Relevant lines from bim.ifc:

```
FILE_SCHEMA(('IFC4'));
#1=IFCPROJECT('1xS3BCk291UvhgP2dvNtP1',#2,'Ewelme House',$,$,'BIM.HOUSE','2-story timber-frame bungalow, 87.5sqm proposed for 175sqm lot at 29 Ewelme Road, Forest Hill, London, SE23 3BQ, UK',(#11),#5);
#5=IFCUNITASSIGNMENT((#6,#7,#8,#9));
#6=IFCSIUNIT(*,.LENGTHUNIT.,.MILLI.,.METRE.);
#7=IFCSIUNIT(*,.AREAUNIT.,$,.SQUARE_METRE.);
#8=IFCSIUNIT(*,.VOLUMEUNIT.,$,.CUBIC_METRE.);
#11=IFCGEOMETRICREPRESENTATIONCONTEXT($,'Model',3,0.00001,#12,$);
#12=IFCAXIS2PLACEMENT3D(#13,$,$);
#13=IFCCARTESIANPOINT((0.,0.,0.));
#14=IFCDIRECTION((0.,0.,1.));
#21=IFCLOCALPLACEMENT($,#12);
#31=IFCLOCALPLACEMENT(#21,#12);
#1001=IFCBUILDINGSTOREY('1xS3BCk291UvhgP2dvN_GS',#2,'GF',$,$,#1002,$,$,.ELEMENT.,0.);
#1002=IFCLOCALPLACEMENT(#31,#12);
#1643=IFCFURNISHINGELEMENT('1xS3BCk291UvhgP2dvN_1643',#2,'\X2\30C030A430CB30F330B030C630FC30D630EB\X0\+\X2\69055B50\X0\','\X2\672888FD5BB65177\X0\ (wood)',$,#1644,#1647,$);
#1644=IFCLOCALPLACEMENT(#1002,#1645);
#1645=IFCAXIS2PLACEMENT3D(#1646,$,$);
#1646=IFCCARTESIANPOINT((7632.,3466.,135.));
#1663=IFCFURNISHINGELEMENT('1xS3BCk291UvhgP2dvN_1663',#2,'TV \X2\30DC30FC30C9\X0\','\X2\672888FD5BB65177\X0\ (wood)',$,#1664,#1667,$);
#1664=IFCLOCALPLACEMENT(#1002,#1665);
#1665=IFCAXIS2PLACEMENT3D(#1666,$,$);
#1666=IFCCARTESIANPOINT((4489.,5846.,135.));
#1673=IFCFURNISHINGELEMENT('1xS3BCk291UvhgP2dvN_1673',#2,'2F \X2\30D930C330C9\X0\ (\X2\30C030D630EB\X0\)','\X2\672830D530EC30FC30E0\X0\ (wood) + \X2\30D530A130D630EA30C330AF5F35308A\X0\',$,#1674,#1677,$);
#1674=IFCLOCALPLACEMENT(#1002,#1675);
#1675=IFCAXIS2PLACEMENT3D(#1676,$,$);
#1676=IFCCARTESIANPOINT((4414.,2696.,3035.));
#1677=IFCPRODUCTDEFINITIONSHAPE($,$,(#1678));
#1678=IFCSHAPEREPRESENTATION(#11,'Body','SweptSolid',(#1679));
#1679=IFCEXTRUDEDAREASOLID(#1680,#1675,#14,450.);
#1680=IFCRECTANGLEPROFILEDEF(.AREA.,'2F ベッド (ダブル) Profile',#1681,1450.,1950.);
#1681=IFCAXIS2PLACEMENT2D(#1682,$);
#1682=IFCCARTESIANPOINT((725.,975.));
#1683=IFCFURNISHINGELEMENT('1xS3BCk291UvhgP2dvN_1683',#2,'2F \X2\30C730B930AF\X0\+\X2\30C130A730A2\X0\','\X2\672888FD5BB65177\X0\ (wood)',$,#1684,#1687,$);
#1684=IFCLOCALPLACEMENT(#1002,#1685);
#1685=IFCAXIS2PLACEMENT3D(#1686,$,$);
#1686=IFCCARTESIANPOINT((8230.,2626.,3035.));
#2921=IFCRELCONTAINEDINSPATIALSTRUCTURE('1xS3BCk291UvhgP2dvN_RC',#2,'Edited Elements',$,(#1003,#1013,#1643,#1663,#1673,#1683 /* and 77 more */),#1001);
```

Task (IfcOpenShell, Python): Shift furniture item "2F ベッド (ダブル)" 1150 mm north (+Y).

```python
import ifcopenshell
import ifcopenshell.api.geometry
import ifcopenshell.util.placement
import ifcopenshell.util.unit

model = ifcopenshell.open("bim.ifc")
unit_scale = ifcopenshell.util.unit.calculate_unit_scale(model)

item = model.by_guid("1xS3BCk291UvhgP2dvN_1673")
matrix = ifcopenshell.util.placement.get_local_placement(item.ObjectPlacement)
matrix[1, 3] += 1.15 / unit_scale
ifcopenshell.api.geometry.edit_object_placement(model, product=item, matrix=matrix, is_si=False)

print(ifcopenshell.util.placement.get_local_placement(item.ObjectPlacement).round(3) + 0.0)

model.write("bim_v2.ifc")
```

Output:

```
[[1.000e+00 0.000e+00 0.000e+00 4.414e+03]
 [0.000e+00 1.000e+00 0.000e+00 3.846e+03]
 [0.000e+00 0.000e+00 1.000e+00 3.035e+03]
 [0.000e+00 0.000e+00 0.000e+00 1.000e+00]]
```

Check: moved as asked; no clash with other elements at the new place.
